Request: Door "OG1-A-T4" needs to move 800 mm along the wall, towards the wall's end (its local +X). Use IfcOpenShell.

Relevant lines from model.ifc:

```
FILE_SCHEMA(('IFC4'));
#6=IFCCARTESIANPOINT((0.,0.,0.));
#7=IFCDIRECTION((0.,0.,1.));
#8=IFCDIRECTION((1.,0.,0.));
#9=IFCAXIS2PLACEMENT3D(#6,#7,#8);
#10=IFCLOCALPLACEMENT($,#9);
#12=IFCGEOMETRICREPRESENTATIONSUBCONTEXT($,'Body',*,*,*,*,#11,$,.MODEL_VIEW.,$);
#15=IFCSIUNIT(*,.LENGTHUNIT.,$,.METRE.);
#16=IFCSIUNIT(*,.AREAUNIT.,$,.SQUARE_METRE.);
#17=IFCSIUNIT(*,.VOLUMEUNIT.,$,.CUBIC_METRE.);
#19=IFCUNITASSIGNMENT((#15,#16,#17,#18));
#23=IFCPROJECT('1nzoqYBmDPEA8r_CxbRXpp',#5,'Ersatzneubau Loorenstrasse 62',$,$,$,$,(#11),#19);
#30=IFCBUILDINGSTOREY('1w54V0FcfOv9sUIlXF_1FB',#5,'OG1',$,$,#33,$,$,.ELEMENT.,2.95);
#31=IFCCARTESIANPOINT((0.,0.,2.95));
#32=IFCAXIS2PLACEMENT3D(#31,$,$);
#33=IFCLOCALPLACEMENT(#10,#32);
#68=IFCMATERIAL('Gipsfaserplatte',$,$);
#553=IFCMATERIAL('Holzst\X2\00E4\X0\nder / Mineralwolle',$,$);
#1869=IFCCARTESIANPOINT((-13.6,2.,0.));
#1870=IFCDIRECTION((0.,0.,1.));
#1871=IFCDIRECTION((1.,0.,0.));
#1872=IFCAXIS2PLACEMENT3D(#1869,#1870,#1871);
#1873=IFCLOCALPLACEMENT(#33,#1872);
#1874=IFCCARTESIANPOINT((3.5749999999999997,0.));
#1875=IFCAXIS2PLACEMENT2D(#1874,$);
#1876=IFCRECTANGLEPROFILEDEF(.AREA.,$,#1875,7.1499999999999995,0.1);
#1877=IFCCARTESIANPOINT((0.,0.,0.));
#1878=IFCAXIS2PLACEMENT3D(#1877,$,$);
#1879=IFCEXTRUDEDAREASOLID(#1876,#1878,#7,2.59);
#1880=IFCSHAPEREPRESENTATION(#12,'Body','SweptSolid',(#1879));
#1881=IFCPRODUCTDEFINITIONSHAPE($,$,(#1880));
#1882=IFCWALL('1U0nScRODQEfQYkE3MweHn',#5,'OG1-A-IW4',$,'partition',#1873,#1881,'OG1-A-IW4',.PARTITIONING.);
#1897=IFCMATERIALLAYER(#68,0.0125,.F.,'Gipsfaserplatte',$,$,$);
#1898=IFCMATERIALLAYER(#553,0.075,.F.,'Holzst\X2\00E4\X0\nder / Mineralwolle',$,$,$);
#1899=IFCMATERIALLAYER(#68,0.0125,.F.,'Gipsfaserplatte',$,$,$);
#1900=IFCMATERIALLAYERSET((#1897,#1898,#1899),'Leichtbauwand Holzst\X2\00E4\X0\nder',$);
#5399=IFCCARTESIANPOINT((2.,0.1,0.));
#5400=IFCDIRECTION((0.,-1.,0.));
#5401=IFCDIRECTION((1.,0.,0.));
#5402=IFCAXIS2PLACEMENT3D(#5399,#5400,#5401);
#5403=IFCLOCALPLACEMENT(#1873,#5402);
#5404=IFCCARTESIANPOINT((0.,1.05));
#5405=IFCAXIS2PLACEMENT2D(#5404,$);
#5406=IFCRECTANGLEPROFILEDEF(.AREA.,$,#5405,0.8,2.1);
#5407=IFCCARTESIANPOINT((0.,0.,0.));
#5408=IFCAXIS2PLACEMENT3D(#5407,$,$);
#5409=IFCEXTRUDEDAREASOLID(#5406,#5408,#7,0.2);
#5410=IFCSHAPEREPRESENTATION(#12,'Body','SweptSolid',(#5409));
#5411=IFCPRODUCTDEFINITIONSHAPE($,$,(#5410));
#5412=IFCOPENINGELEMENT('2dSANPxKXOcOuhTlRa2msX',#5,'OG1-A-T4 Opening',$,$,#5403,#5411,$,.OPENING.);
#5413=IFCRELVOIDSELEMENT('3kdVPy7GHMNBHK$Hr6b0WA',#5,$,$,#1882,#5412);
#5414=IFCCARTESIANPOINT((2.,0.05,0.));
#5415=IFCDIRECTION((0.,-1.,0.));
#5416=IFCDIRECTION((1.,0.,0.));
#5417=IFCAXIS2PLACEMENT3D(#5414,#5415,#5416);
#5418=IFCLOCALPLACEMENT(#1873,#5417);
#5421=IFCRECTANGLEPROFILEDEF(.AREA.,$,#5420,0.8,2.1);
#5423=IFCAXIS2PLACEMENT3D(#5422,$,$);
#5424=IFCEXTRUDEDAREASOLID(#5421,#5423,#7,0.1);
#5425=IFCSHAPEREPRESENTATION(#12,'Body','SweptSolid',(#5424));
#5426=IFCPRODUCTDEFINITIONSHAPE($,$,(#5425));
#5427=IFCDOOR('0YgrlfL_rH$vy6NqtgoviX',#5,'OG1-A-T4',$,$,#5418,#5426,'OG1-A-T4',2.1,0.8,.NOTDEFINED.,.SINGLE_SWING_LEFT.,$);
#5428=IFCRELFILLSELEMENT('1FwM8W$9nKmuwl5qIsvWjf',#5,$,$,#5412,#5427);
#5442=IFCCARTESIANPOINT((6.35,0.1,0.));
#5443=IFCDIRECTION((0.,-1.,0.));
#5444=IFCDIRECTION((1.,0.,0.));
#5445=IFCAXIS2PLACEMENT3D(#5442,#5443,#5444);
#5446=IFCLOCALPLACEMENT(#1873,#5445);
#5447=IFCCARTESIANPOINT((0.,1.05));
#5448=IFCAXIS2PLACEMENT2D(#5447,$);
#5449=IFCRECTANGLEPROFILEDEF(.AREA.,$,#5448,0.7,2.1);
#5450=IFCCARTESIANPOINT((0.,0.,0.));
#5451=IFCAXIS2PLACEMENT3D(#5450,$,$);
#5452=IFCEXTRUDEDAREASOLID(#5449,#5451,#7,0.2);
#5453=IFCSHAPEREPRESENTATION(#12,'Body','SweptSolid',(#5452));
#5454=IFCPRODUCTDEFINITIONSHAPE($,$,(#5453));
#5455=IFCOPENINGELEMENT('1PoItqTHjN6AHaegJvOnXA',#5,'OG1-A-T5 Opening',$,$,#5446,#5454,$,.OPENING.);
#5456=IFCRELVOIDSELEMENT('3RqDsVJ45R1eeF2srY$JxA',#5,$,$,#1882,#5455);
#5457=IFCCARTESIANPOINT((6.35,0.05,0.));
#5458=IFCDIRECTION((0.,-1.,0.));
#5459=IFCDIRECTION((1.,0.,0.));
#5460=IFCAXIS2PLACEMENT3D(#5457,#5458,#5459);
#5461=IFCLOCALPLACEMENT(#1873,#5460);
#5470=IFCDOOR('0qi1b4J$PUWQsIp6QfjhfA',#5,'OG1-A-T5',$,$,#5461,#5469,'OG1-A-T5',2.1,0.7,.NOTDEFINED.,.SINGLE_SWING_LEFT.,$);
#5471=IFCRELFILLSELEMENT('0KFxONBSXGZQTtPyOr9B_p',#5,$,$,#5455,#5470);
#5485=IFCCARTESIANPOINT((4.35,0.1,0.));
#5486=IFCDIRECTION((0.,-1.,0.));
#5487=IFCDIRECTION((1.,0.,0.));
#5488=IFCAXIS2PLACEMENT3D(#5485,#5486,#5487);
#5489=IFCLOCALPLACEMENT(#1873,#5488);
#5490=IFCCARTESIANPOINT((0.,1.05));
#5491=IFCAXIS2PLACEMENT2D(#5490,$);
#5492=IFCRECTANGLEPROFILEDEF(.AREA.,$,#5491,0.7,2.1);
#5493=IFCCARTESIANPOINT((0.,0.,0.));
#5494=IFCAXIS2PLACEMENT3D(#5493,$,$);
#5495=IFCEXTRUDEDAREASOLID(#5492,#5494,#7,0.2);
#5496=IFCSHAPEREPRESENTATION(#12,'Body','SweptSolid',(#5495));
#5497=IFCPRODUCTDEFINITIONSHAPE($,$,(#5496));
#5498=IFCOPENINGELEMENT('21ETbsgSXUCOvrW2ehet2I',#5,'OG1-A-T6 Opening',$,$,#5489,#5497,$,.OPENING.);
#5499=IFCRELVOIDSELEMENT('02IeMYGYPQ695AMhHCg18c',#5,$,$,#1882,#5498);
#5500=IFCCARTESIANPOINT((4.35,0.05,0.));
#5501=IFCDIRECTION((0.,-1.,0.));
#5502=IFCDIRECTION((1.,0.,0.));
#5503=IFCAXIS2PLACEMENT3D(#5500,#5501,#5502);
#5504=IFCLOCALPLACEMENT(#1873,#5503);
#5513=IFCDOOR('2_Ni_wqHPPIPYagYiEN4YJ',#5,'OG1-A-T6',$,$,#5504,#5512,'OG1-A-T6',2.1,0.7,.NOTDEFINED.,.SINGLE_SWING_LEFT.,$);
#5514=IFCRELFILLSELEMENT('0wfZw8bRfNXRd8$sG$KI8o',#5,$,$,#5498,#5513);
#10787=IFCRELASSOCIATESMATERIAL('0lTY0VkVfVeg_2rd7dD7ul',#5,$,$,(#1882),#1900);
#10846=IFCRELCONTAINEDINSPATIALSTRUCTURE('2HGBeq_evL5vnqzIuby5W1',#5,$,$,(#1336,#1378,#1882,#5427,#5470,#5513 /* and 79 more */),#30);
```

```python
import ifcopenshell
import ifcopenshell.api.geometry
import ifcopenshell.util.placement
import ifcopenshell.util.unit

model = ifcopenshell.open("model.ifc")
unit_scale = ifcopenshell.util.unit.calculate_unit_scale(model)

door = model.by_guid("0YgrlfL_rH$vy6NqtgoviX")
opening = door.FillsVoids[0].RelatingOpeningElement
wall = opening.VoidsElements[0].RelatingBuildingElement

wall_matrix = ifcopenshell.util.placement.get_local_placement(wall.ObjectPlacement)
shift = wall_matrix[:3, 0] * 0.8 / unit_scale
before = ifcopenshell.util.placement.get_local_placement(door.ObjectPlacement)[:3, 3].copy()

# The door is not placed relative to its opening, so move both.
for product in (opening, door):
    matrix = ifcopenshell.util.placement.get_local_placement(product.ObjectPlacement)
    matrix[:3, 3] += shift
    ifcopenshell.api.geometry.edit_object_placement(model, product=product, matrix=matrix, is_si=False)

after = ifcopenshell.util.placement.get_local_placement(door.ObjectPlacement)[:3, 3]
print("door moved by", (after - before).round(3) + 0.0)

model.write("model_edited.ifc")
```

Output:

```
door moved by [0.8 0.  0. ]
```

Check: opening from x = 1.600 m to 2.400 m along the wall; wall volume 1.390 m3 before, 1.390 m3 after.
